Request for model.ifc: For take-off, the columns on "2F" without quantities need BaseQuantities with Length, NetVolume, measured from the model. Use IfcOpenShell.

First a look at what the model holds.

```python
import ifcopenshell
import ifcopenshell.util.element
import ifcopenshell.util.unit

model = ifcopenshell.open("model.ifc")
print(model.schema)
for unit_type in ("LENGTHUNIT", "AREAUNIT", "VOLUMEUNIT"):
    print(unit_type, ifcopenshell.util.unit.calculate_unit_scale(model, unit_type))
storey = next(s for s in model.by_type("IfcBuildingStorey") if s.Name == "2F")
columns = [e for e in ifcopenshell.util.element.get_decomposition(storey) if e.is_a("IfcColumn")]
for e in sorted(columns, key=lambda e: e.id()):
    print(e.id(), e.is_a(), e.Name, list(ifcopenshell.util.element.get_psets(e, qtos_only=True)), sep=" | ")
```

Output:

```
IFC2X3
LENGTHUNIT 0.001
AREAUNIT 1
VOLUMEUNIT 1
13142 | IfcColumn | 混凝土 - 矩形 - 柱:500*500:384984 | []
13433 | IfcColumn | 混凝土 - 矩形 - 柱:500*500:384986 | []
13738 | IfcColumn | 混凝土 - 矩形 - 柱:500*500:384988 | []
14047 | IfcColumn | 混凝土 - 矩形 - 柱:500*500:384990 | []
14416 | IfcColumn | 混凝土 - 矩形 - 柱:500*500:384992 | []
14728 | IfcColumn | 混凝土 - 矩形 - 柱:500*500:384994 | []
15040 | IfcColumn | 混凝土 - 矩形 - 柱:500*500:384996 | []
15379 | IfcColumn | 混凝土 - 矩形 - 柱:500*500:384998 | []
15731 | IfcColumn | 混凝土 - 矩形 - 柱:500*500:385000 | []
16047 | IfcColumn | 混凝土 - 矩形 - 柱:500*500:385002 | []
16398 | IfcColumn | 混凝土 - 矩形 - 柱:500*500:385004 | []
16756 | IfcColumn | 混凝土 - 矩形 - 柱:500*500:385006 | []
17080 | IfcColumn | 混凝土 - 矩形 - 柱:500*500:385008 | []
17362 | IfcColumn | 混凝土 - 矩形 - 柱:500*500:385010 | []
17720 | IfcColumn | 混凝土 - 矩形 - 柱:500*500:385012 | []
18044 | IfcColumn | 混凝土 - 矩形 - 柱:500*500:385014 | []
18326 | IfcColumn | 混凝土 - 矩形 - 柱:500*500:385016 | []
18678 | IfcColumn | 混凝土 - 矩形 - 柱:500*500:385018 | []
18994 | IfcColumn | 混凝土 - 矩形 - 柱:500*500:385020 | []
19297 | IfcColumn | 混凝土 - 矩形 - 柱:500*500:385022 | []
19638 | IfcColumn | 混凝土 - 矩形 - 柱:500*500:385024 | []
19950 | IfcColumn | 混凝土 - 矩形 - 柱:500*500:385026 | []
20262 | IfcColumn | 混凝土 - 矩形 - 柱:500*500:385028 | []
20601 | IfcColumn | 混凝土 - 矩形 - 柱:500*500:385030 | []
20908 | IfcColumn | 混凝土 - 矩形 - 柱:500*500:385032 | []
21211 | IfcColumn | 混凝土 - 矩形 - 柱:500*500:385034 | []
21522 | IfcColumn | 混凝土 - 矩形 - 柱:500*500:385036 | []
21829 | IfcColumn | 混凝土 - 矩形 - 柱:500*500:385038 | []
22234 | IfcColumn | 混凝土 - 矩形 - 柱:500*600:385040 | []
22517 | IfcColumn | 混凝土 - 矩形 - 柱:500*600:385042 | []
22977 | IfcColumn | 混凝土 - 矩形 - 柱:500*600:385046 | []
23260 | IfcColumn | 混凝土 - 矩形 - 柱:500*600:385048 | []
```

```python
import ifcopenshell
import ifcopenshell.api.pset
import ifcopenshell.geom
import ifcopenshell.util.element
import ifcopenshell.util.shape
import ifcopenshell.util.unit

model = ifcopenshell.open("model.ifc")
unit_scale = ifcopenshell.util.unit.calculate_unit_scale(model)
volume_scale = ifcopenshell.util.unit.calculate_unit_scale(model, "VOLUMEUNIT")
settings = ifcopenshell.geom.settings()

storey = next(s for s in model.by_type("IfcBuildingStorey") if s.Name == "2F")
columns = [e for e in ifcopenshell.util.element.get_decomposition(storey) if e.is_a("IfcColumn")]

for e in sorted(columns, key=lambda e: e.id()):
    if ifcopenshell.util.element.get_psets(e, qtos_only=True, should_inherit=False):
        continue
    # Geometry comes back in metres, in the element's own axes.
    shape = ifcopenshell.geom.create_shape(settings, e)
    values = {
        "Length": ifcopenshell.util.shape.get_z(shape.geometry) / unit_scale,
        "NetVolume": ifcopenshell.util.shape.get_volume(shape.geometry) / volume_scale,
    }
    qto = ifcopenshell.api.pset.add_qto(model, product=e, name="BaseQuantities")
    ifcopenshell.api.pset.edit_qto(model, qto=qto, properties=values)
    print(e.id(), {k: round(v, 3) for k, v in values.items()})

model.write("model_edited.ifc")
```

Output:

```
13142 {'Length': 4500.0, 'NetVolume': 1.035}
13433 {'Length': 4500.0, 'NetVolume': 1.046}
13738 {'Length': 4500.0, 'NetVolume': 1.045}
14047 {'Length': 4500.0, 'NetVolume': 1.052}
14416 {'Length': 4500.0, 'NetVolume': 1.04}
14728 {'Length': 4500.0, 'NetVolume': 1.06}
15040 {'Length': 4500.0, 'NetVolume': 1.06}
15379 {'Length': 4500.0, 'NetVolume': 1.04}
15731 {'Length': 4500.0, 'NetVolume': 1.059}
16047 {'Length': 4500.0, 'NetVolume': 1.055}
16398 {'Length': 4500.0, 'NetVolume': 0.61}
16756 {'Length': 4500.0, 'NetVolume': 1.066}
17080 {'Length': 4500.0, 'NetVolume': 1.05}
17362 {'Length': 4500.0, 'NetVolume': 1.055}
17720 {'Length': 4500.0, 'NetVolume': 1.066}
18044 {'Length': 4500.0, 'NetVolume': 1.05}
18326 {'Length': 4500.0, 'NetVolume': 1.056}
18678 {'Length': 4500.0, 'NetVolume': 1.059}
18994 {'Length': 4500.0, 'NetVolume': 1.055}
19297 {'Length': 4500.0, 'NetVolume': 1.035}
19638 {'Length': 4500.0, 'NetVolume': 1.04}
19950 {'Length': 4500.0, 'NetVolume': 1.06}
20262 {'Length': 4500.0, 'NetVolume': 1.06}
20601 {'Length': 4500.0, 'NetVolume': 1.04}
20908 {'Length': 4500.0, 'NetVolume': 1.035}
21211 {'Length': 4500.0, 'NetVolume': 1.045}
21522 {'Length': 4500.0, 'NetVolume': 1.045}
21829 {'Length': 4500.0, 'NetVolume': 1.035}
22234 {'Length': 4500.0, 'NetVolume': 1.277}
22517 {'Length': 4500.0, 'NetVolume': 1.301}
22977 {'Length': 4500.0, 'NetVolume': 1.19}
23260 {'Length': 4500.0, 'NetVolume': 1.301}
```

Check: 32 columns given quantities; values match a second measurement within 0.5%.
